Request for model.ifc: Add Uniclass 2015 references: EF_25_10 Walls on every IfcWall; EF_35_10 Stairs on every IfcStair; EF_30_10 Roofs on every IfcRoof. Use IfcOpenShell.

First a look at what the model holds.

```python
import ifcopenshell

model = ifcopenshell.open("model.ifc")
print(model.schema)
print("classifications:", [c.Name for c in model.by_type("IfcClassification")])
for ifc_class in ("IfcDoor", "IfcRoof", "IfcStair", "IfcWall", "IfcWindow"):
    print(ifc_class, len(model.by_type(ifc_class)))
```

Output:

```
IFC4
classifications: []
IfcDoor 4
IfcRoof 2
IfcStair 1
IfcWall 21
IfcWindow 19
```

```python
import ifcopenshell
import ifcopenshell.api.classification

model = ifcopenshell.open("model.ifc")

system = ifcopenshell.api.classification.add_classification(model, classification="Uniclass 2015")

codes = {
    "IfcWall": ("EF_25_10", "Walls"),
    "IfcStair": ("EF_35_10", "Stairs"),
    "IfcRoof": ("EF_30_10", "Roofs"),
}
for ifc_class, (code, name) in codes.items():
    products = model.by_type(ifc_class)
    ifcopenshell.api.classification.add_reference(
        model, products=products, classification=system, identification=code, name=name
    )
    print(code, len(products))

model.write("model_updated.ifc")
```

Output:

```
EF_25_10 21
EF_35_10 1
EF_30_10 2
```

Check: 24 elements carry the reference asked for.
